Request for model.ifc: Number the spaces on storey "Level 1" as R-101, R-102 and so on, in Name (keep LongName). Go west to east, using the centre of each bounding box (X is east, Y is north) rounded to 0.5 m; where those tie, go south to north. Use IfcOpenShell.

First a look at what the model holds.

```python
import ifcopenshell
import ifcopenshell.util.element
import ifcopenshell.util.placement

model = ifcopenshell.open("model.ifc")
print(model.schema)
storey = next(s for s in model.by_type("IfcBuildingStorey") if s.Name == "Level 1")
spaces = [e for e in ifcopenshell.util.element.get_decomposition(storey) if e.is_a("IfcSpace")]
for e in sorted(spaces, key=lambda e: e.id()):
    origin = ifcopenshell.util.placement.get_local_placement(e.ObjectPlacement)[:3, 3]
    print(e.id(), e.Name, e.LongName, origin.round(2) + 0.0, sep=" | ")
```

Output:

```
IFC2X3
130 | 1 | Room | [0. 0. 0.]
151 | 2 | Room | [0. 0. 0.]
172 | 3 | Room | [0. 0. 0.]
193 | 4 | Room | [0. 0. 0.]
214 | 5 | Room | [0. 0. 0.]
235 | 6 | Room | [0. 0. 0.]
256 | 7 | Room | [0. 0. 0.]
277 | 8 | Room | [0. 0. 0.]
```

```python
import ifcopenshell
import ifcopenshell.geom
import ifcopenshell.util.element
import ifcopenshell.util.shape

model = ifcopenshell.open("model.ifc")
settings = ifcopenshell.geom.settings()
settings.set("use-world-coords", True)


def centre(element):
    shape = ifcopenshell.geom.create_shape(settings, element)
    return ifcopenshell.util.shape.get_bbox_centroid(shape.geometry)


storey = next(s for s in model.by_type("IfcBuildingStorey") if s.Name == "Level 1")
spaces = [e for e in ifcopenshell.util.element.get_decomposition(storey) if e.is_a("IfcSpace")]

# Insertion points can sit at a corner or the storey origin, so sort by the geometry (in metres).
centres = {e: centre(e) for e in spaces}
spaces.sort(key=lambda e: (round(centres[e][0] / 0.5), centres[e][1]))

for i, e in enumerate(spaces, start=1):
    number = f"R-1{i:02d}"
    e.Name = number
    print(e.id(), number)

model.write("model_edited.ifc")
```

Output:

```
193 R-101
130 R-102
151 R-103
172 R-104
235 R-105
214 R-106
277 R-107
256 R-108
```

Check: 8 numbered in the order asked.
